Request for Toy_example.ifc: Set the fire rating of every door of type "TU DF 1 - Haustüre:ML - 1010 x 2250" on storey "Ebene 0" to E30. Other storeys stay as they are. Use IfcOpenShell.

First a look at what the model holds.

```python
import ifcopenshell
import ifcopenshell.util.element

model = ifcopenshell.open("Toy_example.ifc")
print(model.schema)
storey = next(s for s in model.by_type("IfcBuildingStorey") if s.Name == "Ebene 0")
doors = [e for e in ifcopenshell.util.element.get_decomposition(storey) if e.is_a("IfcDoor")]
seen = {}
for e in doors:
    element_type = ifcopenshell.util.element.get_type(e)
    key = (element_type.Name if element_type != e and element_type else None, ifcopenshell.util.element.get_pset(e, "Pset_DoorCommon", "FireRating"))
    seen[key] = seen.get(key, 0) + 1
for (name, value), count in sorted(seen.items(), key=str):
    print(count, "x", name, "|", value)
```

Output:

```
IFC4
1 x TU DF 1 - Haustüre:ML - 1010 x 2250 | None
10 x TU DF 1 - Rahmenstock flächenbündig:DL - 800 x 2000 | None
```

```python
import ifcopenshell
import ifcopenshell.api.pset
import ifcopenshell.util.element

model = ifcopenshell.open("Toy_example.ifc")

storey = next(s for s in model.by_type("IfcBuildingStorey") if s.Name == "Ebene 0")
doors = [e for e in ifcopenshell.util.element.get_decomposition(storey) if e.is_a("IfcDoor")]

count = 0
for e in doors:
    element_type = ifcopenshell.util.element.get_type(e)
    if element_type in (None, e) or element_type.Name != "TU DF 1 - Haustüre:ML - 1010 x 2250":
        continue
    # add_pset returns the element's existing set when there is one.
    pset = ifcopenshell.api.pset.add_pset(model, product=e, name="Pset_DoorCommon")
    ifcopenshell.api.pset.edit_pset(model, pset=pset, properties={"FireRating": "E30"})
    count += 1

print(count, "doors updated")

model.write("Toy_example_edited.ifc")
```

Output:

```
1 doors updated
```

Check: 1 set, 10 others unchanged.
